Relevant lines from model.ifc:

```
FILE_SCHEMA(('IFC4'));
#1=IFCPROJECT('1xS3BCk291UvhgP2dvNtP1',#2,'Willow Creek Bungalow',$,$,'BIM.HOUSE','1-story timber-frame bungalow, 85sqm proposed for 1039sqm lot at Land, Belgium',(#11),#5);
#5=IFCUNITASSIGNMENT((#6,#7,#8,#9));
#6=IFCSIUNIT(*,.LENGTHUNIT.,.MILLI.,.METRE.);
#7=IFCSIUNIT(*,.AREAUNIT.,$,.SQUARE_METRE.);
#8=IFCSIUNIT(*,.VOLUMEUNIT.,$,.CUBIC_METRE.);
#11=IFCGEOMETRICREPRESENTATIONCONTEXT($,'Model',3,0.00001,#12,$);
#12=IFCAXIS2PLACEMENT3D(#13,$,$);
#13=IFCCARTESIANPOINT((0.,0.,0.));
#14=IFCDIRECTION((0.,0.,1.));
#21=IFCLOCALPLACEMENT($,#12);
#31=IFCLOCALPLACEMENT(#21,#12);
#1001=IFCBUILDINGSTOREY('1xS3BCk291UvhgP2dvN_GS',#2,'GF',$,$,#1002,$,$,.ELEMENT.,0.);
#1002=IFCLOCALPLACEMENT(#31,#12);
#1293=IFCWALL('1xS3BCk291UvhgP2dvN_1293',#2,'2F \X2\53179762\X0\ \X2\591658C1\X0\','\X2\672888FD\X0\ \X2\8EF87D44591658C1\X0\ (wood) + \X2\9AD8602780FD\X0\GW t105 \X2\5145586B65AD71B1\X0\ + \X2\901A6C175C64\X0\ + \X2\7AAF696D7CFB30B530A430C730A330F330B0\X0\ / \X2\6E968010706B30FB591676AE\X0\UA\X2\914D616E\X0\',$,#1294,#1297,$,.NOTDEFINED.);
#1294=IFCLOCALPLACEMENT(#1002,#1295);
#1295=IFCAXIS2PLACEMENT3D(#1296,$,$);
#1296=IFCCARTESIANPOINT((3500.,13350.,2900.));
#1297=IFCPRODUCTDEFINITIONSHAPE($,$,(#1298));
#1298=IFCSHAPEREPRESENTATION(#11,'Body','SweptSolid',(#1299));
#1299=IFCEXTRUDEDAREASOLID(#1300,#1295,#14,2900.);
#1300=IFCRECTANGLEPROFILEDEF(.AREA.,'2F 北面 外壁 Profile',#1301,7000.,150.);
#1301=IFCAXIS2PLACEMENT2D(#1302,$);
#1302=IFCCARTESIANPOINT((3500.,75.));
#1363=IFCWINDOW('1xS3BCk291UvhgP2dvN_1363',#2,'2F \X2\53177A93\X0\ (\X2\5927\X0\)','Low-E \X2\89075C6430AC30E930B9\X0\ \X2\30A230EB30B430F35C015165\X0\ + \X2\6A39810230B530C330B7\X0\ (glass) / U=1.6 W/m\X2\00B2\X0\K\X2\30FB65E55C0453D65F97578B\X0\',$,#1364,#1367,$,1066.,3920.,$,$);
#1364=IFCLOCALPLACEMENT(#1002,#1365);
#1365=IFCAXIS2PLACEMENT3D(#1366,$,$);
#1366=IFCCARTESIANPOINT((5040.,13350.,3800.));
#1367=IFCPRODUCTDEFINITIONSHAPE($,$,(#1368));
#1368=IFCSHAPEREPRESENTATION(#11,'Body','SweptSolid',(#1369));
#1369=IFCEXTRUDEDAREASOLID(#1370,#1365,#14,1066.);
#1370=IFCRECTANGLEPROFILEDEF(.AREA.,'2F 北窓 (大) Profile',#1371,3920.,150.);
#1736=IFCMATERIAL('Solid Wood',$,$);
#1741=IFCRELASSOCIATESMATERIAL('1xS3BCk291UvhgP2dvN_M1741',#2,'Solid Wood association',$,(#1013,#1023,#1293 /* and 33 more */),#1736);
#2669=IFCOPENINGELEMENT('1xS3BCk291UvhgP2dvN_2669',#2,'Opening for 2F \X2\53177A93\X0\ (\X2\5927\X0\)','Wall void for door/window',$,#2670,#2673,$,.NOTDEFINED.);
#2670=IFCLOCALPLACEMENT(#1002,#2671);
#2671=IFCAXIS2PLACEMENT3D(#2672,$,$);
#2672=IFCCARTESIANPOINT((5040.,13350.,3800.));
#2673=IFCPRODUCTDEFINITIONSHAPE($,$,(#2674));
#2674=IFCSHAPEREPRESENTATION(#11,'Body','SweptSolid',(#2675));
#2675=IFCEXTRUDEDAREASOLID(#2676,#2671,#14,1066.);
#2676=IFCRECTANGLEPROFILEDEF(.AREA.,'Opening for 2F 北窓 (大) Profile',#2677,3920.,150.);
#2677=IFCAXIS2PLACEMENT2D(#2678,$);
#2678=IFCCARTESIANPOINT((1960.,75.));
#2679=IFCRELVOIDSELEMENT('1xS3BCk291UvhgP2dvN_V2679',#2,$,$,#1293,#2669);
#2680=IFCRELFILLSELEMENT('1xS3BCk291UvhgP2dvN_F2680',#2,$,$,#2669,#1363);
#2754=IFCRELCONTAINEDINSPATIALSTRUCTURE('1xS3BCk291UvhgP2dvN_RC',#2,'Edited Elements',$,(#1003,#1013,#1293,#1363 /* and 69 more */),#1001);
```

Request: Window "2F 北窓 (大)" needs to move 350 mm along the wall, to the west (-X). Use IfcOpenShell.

```python
import ifcopenshell
import ifcopenshell.api.geometry
import ifcopenshell.util.placement
import ifcopenshell.util.unit

model = ifcopenshell.open("model.ifc")
unit_scale = ifcopenshell.util.unit.calculate_unit_scale(model)

window = model.by_id(1363)
opening = window.FillsVoids[0].RelatingOpeningElement
wall = opening.VoidsElements[0].RelatingBuildingElement

wall_matrix = ifcopenshell.util.placement.get_local_placement(wall.ObjectPlacement)
shift = wall_matrix[:3, 0] * -0.35 / unit_scale
before = ifcopenshell.util.placement.get_local_placement(window.ObjectPlacement)[:3, 3].copy()

# The window is not placed relative to its opening, so move both.
for product in (opening, window):
    matrix = ifcopenshell.util.placement.get_local_placement(product.ObjectPlacement)
    matrix[:3, 3] += shift
    ifcopenshell.api.geometry.edit_object_placement(model, product=product, matrix=matrix, is_si=False)

after = ifcopenshell.util.placement.get_local_placement(window.ObjectPlacement)[:3, 3]
print("window moved by", (after - before).round(3) + 0.0)

model.write("model_v2.ifc")
```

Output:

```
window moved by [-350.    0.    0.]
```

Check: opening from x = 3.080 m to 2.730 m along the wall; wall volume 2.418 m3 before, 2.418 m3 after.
